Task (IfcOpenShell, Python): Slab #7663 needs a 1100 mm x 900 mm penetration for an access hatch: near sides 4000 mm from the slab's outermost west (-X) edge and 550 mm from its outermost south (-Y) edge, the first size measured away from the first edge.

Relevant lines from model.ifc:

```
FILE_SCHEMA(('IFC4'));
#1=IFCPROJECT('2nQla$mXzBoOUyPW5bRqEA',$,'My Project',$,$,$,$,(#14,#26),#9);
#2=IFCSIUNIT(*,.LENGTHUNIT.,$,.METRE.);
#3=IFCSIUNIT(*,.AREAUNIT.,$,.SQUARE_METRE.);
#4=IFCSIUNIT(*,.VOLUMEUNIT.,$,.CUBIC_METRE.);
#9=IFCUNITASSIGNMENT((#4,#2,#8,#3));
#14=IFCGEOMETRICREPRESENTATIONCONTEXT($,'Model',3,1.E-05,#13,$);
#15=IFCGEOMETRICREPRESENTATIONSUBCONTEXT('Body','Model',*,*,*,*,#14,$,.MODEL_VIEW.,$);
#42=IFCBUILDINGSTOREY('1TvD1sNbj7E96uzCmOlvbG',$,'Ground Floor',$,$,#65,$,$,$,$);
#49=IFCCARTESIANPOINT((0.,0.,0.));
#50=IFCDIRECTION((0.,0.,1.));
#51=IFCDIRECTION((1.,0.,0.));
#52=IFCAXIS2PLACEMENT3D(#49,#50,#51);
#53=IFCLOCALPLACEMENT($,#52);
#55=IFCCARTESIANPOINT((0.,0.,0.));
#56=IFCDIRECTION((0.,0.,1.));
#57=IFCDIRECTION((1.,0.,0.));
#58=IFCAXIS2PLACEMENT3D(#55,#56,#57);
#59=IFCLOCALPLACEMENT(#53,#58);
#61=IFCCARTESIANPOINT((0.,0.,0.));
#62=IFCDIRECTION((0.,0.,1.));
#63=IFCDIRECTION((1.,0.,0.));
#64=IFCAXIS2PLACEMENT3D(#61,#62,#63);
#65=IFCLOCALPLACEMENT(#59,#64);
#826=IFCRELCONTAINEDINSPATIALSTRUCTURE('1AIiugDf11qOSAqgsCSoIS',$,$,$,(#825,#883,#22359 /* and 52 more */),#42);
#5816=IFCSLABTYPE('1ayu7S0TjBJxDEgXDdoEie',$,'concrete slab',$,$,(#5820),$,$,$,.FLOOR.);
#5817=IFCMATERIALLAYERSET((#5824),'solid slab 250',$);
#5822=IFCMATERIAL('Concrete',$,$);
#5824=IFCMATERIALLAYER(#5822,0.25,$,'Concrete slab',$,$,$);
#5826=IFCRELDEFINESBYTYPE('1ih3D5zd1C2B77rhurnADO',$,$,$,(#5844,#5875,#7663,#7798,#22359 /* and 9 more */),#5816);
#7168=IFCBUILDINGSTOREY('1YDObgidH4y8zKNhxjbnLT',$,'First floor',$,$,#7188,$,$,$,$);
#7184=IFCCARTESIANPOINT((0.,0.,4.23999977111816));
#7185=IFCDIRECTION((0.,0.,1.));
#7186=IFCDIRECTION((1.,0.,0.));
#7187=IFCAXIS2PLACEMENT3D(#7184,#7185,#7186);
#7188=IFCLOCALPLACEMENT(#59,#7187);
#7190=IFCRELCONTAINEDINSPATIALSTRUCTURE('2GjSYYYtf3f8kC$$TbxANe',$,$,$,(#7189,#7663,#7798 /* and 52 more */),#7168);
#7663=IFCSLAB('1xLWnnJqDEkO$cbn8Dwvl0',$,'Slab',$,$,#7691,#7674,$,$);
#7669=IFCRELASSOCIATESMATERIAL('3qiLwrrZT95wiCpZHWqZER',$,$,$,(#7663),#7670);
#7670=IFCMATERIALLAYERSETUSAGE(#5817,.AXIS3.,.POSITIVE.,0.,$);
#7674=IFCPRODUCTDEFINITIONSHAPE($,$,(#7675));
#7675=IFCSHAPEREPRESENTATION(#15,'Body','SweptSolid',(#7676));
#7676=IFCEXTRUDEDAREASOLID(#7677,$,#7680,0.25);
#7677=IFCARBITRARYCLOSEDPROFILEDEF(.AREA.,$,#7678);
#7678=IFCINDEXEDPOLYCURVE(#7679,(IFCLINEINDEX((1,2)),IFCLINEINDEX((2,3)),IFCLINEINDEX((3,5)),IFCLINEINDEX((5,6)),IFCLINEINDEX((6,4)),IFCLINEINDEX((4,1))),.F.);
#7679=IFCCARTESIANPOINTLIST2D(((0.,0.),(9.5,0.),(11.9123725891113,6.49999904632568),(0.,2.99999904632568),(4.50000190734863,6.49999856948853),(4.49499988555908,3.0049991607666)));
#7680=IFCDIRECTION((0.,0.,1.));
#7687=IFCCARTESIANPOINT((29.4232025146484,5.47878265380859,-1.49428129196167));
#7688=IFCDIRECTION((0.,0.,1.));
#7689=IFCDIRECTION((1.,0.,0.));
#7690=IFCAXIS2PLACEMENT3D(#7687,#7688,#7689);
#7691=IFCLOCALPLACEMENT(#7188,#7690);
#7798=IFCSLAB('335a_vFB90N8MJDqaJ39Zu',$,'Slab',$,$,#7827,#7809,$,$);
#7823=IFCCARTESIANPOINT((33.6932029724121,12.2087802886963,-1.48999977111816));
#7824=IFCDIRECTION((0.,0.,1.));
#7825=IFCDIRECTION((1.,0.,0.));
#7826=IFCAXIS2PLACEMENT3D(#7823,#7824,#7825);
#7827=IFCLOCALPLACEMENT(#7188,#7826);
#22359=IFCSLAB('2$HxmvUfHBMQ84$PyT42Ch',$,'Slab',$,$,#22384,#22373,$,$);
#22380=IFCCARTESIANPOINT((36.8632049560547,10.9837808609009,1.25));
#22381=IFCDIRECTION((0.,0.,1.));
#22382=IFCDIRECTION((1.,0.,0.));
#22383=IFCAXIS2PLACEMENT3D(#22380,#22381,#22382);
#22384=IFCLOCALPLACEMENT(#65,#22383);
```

```python
import numpy as np
import ifcopenshell
import ifcopenshell.api.feature
import ifcopenshell.api.geometry
import ifcopenshell.api.root
import ifcopenshell.geom
import ifcopenshell.util.placement
import ifcopenshell.util.representation
import ifcopenshell.util.shape
import ifcopenshell.util.unit

model = ifcopenshell.open("model.ifc")
unit_scale = ifcopenshell.util.unit.calculate_unit_scale(model)
settings = ifcopenshell.geom.settings()


def volume(element):
    """Net volume in cubic metres, openings subtracted."""
    shape = ifcopenshell.geom.create_shape(settings, element)
    return ifcopenshell.util.shape.get_volume(shape.geometry)


slab = model.by_guid("1xLWnnJqDEkO$cbn8Dwvl0")
before = volume(slab)

# Extent in the slab's own axes, in metres. The edges named are its -X and -Y sides.
slab_shape = ifcopenshell.geom.create_shape(settings, slab)
vertices = ifcopenshell.util.shape.get_vertices(slab_shape.geometry)
x_min, y_min, bottom = vertices.min(axis=0)
top = vertices[:, 2].max()

opening = ifcopenshell.api.root.create_entity(model, ifc_class="IfcOpeningElement", name="Access hatch opening", predefined_type="OPENING")
context = ifcopenshell.util.representation.get_context(model, "Model", "Body", "MODEL_VIEW")
width, depth = 1.1, 0.9
outline = [(0.0, 0.0), (width, 0.0), (width, depth), (0.0, depth), (0.0, 0.0)]
# Overshoot both faces by 50 mm so the cut is clean.
shape = ifcopenshell.api.geometry.add_slab_representation(
    model, context=context, depth=top - bottom + 0.1, polyline=outline
)
ifcopenshell.api.geometry.assign_representation(model, product=opening, representation=shape)

matrix = ifcopenshell.util.placement.get_local_placement(slab.ObjectPlacement)
matrix[:, 3] = matrix @ np.append(np.array([x_min + 4, y_min + 0.55, bottom - 0.05]) / unit_scale, 1.0)
ifcopenshell.api.geometry.edit_object_placement(model, product=opening, matrix=matrix, is_si=False)
ifcopenshell.api.feature.add_feature(model, feature=opening, element=slab)

after = volume(slab)

print(f"slab volume {before:.3f} -> {after:.3f} m3")

model.write("model-out.ifc")
```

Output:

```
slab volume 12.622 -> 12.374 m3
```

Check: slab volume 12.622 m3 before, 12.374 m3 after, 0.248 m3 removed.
